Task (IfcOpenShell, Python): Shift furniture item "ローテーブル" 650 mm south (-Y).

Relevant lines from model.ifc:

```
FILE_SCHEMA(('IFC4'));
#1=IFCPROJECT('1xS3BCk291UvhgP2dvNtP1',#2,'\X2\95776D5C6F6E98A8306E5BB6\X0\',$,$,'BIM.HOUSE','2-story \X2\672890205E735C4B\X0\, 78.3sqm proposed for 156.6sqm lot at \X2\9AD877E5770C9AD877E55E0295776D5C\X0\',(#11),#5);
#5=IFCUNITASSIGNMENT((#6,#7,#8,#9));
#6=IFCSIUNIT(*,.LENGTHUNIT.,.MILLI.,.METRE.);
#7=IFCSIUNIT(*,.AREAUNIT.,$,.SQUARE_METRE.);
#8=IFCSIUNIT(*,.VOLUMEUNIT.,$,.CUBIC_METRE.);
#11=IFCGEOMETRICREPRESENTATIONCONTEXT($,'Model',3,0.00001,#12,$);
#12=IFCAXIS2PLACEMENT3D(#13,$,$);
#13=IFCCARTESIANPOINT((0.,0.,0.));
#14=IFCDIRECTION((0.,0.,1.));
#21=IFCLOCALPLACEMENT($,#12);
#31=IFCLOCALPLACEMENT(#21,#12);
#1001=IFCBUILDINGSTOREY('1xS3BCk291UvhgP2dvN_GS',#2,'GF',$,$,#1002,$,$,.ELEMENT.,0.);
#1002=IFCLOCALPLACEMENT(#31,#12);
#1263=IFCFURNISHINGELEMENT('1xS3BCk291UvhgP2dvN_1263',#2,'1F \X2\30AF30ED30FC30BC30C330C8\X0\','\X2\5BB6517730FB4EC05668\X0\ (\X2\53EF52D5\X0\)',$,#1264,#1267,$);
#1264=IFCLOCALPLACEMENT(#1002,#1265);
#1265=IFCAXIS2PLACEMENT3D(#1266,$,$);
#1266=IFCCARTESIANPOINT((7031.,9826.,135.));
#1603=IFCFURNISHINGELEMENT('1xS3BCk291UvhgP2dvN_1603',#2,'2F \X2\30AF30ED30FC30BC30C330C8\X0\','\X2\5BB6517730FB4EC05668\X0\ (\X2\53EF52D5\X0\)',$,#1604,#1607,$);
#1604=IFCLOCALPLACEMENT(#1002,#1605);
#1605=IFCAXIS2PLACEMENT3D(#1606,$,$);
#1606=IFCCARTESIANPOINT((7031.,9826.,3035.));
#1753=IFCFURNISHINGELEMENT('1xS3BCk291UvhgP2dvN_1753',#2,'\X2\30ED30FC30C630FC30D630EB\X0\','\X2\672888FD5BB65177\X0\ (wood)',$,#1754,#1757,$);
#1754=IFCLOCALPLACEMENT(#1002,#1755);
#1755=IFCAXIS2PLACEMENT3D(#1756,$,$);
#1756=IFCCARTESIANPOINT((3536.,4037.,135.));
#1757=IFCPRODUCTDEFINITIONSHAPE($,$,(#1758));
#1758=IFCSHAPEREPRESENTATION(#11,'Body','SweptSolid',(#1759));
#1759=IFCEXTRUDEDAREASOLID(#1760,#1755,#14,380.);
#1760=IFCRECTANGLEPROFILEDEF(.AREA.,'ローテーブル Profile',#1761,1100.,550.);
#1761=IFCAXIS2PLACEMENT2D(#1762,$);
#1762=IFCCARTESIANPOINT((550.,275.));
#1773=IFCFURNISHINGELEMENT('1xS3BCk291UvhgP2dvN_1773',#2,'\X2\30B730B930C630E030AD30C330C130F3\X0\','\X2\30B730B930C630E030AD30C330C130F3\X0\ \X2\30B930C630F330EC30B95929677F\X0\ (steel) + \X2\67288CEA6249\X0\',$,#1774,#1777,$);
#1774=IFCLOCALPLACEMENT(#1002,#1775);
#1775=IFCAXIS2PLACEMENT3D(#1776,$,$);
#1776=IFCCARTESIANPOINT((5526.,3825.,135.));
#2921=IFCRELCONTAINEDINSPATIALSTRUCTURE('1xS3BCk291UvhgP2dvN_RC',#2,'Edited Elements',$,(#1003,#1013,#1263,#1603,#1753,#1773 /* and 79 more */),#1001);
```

```python
import ifcopenshell
import ifcopenshell.api.geometry
import ifcopenshell.util.placement
import ifcopenshell.util.unit

model = ifcopenshell.open("model.ifc")
unit_scale = ifcopenshell.util.unit.calculate_unit_scale(model)

item = model.by_guid("1xS3BCk291UvhgP2dvN_1753")
matrix = ifcopenshell.util.placement.get_local_placement(item.ObjectPlacement)
matrix[1, 3] -= 0.65 / unit_scale
ifcopenshell.api.geometry.edit_object_placement(model, product=item, matrix=matrix, is_si=False)

print(ifcopenshell.util.placement.get_local_placement(item.ObjectPlacement).round(3) + 0.0)

model.write("model_rev.ifc")
```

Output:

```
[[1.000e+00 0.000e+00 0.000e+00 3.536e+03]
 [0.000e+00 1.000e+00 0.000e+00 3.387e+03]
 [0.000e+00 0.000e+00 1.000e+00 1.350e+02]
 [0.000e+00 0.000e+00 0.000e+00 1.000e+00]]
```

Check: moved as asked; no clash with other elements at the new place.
